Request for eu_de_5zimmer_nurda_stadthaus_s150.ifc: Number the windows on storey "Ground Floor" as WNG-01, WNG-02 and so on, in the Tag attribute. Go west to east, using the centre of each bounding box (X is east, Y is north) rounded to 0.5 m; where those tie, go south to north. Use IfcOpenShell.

First a look at what the model holds.

```python
import ifcopenshell
import ifcopenshell.util.element
import ifcopenshell.util.placement

model = ifcopenshell.open("eu_de_5zimmer_nurda_stadthaus_s150.ifc")
print(model.schema)
storey = next(s for s in model.by_type("IfcBuildingStorey") if s.Name == "Ground Floor")
windows = [e for e in ifcopenshell.util.element.get_decomposition(storey) if e.is_a("IfcWindow")]
for e in sorted(windows, key=lambda e: e.id()):
    origin = ifcopenshell.util.placement.get_local_placement(e.ObjectPlacement)[:3, 3]
    print(e.id(), e.Tag, e.Name, origin.round(2) + 0.0, sep=" | ")
```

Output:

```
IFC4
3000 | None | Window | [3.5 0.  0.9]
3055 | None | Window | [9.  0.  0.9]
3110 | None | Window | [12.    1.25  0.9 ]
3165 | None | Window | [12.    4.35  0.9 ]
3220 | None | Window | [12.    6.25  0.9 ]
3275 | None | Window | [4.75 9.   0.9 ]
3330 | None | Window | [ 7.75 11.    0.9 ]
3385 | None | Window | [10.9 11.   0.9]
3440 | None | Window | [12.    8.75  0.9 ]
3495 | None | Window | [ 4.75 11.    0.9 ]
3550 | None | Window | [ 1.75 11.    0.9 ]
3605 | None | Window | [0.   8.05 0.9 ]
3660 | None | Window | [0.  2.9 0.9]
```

```python
import ifcopenshell
import ifcopenshell.geom
import ifcopenshell.util.element
import ifcopenshell.util.shape

model = ifcopenshell.open("eu_de_5zimmer_nurda_stadthaus_s150.ifc")
settings = ifcopenshell.geom.settings()
settings.set("use-world-coords", True)


def centre(element):
    shape = ifcopenshell.geom.create_shape(settings, element)
    return ifcopenshell.util.shape.get_bbox_centroid(shape.geometry)


storey = next(s for s in model.by_type("IfcBuildingStorey") if s.Name == "Ground Floor")
windows = [e for e in ifcopenshell.util.element.get_decomposition(storey) if e.is_a("IfcWindow")]

# Insertion points can sit at a corner or the storey origin, so sort by the geometry (in metres).
centres = {e: centre(e) for e in windows}
windows.sort(key=lambda e: (round(centres[e][0] / 0.5), centres[e][1]))

for i, e in enumerate(windows, start=1):
    number = f"WNG-{i:02d}"
    e.Tag = number
    print(e.id(), number)

model.write("eu_de_5zimmer_nurda_stadthaus_s150_updated.ifc")
```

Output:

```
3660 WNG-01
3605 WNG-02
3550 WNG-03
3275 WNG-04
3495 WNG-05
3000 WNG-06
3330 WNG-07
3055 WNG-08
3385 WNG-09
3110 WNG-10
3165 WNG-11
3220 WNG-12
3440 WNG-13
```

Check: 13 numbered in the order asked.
